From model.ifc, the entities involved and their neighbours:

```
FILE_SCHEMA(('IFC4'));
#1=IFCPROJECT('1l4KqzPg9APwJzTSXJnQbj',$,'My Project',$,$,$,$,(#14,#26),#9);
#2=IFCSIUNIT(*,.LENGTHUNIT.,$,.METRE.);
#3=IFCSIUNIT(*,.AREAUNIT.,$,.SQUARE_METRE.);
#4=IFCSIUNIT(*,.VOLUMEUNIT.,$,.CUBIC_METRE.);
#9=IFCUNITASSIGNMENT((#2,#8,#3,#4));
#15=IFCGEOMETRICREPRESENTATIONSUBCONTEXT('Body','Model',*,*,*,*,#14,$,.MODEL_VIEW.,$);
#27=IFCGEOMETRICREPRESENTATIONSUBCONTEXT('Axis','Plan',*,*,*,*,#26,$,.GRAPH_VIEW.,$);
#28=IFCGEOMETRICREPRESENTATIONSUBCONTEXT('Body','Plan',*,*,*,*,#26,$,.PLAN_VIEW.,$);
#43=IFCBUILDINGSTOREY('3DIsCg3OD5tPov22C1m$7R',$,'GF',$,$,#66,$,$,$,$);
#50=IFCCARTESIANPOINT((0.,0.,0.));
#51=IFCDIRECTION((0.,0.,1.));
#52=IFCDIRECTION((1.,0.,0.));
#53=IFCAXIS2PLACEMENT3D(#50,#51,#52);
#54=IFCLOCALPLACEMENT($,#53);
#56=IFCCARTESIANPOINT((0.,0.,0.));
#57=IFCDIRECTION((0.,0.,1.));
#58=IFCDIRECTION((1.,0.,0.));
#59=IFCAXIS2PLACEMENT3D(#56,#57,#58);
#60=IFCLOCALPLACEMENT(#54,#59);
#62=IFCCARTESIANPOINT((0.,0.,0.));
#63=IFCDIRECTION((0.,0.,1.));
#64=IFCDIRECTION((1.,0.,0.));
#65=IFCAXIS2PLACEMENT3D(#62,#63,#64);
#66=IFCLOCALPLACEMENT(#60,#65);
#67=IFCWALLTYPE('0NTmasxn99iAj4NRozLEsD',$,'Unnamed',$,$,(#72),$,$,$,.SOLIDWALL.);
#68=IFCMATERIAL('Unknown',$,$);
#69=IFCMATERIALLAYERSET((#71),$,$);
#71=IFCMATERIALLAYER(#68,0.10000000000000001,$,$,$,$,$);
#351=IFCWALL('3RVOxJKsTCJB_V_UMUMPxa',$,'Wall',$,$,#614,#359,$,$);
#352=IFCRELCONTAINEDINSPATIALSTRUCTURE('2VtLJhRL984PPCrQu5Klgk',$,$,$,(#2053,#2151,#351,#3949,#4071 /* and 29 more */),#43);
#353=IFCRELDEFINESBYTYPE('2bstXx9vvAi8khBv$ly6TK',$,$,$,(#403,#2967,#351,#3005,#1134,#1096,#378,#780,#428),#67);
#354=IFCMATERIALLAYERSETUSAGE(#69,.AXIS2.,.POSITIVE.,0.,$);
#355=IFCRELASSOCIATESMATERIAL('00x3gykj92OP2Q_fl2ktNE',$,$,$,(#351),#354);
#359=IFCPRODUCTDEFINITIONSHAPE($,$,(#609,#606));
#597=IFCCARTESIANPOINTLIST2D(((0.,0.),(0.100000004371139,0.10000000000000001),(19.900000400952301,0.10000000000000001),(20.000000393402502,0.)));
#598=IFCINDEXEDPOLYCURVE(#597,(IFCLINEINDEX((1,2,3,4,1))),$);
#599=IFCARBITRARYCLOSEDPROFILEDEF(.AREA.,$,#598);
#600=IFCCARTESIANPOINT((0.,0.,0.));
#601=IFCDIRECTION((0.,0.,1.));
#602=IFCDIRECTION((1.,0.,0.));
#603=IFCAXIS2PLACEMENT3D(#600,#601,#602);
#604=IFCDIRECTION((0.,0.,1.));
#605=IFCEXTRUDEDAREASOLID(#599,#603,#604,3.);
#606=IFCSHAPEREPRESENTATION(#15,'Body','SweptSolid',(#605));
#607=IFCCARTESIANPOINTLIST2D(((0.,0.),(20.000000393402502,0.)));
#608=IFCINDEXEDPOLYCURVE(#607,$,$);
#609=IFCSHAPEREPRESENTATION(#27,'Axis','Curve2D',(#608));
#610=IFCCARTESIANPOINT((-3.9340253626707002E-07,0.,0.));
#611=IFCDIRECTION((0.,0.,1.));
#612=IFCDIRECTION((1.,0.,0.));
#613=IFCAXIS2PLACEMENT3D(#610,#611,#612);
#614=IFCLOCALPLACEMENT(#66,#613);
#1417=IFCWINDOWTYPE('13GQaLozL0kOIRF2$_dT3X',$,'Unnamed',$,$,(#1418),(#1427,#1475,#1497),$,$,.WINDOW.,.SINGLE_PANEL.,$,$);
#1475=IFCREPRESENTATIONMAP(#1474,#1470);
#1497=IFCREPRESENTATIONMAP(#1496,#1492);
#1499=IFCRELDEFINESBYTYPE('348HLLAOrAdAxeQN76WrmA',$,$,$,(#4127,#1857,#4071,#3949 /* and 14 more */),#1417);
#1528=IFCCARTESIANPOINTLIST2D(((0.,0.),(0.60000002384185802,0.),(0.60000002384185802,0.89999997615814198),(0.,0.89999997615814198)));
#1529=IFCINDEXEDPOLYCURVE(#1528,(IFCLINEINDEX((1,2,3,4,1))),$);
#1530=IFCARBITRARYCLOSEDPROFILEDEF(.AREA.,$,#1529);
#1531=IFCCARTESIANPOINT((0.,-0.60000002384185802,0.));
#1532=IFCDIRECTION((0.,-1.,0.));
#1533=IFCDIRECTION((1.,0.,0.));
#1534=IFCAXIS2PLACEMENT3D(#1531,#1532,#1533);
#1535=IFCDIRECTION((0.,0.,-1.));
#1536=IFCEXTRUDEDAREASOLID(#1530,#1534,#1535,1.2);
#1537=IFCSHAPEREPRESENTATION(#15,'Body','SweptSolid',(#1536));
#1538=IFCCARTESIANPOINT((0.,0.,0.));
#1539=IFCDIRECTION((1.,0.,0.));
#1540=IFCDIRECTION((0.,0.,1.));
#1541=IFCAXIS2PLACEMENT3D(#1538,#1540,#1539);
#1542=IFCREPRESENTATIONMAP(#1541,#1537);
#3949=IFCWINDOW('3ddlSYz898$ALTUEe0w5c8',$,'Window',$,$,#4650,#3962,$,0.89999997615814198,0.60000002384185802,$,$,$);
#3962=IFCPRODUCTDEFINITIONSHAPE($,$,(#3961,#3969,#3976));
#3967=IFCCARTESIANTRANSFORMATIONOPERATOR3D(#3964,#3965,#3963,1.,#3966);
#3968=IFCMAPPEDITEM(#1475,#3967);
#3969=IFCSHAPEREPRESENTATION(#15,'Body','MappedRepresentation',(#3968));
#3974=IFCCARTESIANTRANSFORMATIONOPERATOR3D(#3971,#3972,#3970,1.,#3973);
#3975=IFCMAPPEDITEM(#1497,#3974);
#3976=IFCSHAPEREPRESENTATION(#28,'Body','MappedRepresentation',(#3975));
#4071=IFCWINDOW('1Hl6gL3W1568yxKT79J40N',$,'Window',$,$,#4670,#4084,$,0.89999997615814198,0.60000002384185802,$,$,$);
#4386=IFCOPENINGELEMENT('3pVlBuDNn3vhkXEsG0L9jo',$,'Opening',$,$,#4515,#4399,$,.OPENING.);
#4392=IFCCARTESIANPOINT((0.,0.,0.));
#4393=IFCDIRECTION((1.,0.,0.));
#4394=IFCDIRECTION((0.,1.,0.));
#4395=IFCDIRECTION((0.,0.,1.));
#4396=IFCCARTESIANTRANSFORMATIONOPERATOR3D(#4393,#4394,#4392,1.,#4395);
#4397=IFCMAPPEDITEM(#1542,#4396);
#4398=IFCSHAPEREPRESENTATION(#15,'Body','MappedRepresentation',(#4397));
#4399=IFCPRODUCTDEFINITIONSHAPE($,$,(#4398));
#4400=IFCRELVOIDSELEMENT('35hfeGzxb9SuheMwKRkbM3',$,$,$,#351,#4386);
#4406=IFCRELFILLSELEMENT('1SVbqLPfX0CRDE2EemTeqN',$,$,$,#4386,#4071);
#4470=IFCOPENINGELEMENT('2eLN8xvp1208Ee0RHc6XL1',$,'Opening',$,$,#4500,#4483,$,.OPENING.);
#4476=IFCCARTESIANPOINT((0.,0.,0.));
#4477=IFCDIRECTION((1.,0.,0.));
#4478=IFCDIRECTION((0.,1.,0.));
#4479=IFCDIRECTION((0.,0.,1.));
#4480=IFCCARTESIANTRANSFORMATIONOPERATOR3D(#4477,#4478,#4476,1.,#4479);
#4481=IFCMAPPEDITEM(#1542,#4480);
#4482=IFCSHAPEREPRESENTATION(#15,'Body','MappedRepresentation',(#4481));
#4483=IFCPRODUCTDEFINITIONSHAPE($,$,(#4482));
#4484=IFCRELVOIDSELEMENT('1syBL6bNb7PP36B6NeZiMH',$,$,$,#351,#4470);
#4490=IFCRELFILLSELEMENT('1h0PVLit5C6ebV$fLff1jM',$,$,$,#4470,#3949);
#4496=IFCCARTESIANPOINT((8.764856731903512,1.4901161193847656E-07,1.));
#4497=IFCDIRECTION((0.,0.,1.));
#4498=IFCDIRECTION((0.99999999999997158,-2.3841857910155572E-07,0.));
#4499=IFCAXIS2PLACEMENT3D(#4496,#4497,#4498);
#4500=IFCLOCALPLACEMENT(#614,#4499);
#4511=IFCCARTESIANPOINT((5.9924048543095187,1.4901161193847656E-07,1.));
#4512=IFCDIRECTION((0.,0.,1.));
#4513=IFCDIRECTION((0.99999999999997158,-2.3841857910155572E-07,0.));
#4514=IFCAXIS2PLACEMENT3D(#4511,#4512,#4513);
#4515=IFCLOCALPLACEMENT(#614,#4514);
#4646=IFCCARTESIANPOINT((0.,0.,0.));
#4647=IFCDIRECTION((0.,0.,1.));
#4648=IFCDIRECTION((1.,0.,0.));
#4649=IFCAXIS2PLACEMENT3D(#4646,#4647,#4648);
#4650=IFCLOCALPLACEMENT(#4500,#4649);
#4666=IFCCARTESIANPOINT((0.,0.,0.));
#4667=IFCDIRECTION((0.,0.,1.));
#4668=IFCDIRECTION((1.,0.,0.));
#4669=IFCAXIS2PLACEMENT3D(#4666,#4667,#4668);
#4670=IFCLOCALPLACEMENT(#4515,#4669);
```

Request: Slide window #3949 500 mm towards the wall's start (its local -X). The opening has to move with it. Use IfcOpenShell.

```python
import ifcopenshell
import ifcopenshell.api.geometry
import ifcopenshell.util.placement

model = ifcopenshell.open("model.ifc")

window = model.by_id(3949)
opening = window.FillsVoids[0].RelatingOpeningElement
wall = opening.VoidsElements[0].RelatingBuildingElement

wall_matrix = ifcopenshell.util.placement.get_local_placement(wall.ObjectPlacement)
shift = wall_matrix[:3, 0] * -0.5
before = ifcopenshell.util.placement.get_local_placement(window.ObjectPlacement)[:3, 3].copy()

# The window is placed relative to its opening, so it follows when the opening moves.
matrix = ifcopenshell.util.placement.get_local_placement(opening.ObjectPlacement)
matrix[:3, 3] += shift
ifcopenshell.api.geometry.edit_object_placement(
    model, product=opening, matrix=matrix, is_si=False, should_transform_children=True
)

after = ifcopenshell.util.placement.get_local_placement(window.ObjectPlacement)[:3, 3]
print("window moved by", (after - before).round(3) + 0.0)

model.write("model_v2.ifc")
```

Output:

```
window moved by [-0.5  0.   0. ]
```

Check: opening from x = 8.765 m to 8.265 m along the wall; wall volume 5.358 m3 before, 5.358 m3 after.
